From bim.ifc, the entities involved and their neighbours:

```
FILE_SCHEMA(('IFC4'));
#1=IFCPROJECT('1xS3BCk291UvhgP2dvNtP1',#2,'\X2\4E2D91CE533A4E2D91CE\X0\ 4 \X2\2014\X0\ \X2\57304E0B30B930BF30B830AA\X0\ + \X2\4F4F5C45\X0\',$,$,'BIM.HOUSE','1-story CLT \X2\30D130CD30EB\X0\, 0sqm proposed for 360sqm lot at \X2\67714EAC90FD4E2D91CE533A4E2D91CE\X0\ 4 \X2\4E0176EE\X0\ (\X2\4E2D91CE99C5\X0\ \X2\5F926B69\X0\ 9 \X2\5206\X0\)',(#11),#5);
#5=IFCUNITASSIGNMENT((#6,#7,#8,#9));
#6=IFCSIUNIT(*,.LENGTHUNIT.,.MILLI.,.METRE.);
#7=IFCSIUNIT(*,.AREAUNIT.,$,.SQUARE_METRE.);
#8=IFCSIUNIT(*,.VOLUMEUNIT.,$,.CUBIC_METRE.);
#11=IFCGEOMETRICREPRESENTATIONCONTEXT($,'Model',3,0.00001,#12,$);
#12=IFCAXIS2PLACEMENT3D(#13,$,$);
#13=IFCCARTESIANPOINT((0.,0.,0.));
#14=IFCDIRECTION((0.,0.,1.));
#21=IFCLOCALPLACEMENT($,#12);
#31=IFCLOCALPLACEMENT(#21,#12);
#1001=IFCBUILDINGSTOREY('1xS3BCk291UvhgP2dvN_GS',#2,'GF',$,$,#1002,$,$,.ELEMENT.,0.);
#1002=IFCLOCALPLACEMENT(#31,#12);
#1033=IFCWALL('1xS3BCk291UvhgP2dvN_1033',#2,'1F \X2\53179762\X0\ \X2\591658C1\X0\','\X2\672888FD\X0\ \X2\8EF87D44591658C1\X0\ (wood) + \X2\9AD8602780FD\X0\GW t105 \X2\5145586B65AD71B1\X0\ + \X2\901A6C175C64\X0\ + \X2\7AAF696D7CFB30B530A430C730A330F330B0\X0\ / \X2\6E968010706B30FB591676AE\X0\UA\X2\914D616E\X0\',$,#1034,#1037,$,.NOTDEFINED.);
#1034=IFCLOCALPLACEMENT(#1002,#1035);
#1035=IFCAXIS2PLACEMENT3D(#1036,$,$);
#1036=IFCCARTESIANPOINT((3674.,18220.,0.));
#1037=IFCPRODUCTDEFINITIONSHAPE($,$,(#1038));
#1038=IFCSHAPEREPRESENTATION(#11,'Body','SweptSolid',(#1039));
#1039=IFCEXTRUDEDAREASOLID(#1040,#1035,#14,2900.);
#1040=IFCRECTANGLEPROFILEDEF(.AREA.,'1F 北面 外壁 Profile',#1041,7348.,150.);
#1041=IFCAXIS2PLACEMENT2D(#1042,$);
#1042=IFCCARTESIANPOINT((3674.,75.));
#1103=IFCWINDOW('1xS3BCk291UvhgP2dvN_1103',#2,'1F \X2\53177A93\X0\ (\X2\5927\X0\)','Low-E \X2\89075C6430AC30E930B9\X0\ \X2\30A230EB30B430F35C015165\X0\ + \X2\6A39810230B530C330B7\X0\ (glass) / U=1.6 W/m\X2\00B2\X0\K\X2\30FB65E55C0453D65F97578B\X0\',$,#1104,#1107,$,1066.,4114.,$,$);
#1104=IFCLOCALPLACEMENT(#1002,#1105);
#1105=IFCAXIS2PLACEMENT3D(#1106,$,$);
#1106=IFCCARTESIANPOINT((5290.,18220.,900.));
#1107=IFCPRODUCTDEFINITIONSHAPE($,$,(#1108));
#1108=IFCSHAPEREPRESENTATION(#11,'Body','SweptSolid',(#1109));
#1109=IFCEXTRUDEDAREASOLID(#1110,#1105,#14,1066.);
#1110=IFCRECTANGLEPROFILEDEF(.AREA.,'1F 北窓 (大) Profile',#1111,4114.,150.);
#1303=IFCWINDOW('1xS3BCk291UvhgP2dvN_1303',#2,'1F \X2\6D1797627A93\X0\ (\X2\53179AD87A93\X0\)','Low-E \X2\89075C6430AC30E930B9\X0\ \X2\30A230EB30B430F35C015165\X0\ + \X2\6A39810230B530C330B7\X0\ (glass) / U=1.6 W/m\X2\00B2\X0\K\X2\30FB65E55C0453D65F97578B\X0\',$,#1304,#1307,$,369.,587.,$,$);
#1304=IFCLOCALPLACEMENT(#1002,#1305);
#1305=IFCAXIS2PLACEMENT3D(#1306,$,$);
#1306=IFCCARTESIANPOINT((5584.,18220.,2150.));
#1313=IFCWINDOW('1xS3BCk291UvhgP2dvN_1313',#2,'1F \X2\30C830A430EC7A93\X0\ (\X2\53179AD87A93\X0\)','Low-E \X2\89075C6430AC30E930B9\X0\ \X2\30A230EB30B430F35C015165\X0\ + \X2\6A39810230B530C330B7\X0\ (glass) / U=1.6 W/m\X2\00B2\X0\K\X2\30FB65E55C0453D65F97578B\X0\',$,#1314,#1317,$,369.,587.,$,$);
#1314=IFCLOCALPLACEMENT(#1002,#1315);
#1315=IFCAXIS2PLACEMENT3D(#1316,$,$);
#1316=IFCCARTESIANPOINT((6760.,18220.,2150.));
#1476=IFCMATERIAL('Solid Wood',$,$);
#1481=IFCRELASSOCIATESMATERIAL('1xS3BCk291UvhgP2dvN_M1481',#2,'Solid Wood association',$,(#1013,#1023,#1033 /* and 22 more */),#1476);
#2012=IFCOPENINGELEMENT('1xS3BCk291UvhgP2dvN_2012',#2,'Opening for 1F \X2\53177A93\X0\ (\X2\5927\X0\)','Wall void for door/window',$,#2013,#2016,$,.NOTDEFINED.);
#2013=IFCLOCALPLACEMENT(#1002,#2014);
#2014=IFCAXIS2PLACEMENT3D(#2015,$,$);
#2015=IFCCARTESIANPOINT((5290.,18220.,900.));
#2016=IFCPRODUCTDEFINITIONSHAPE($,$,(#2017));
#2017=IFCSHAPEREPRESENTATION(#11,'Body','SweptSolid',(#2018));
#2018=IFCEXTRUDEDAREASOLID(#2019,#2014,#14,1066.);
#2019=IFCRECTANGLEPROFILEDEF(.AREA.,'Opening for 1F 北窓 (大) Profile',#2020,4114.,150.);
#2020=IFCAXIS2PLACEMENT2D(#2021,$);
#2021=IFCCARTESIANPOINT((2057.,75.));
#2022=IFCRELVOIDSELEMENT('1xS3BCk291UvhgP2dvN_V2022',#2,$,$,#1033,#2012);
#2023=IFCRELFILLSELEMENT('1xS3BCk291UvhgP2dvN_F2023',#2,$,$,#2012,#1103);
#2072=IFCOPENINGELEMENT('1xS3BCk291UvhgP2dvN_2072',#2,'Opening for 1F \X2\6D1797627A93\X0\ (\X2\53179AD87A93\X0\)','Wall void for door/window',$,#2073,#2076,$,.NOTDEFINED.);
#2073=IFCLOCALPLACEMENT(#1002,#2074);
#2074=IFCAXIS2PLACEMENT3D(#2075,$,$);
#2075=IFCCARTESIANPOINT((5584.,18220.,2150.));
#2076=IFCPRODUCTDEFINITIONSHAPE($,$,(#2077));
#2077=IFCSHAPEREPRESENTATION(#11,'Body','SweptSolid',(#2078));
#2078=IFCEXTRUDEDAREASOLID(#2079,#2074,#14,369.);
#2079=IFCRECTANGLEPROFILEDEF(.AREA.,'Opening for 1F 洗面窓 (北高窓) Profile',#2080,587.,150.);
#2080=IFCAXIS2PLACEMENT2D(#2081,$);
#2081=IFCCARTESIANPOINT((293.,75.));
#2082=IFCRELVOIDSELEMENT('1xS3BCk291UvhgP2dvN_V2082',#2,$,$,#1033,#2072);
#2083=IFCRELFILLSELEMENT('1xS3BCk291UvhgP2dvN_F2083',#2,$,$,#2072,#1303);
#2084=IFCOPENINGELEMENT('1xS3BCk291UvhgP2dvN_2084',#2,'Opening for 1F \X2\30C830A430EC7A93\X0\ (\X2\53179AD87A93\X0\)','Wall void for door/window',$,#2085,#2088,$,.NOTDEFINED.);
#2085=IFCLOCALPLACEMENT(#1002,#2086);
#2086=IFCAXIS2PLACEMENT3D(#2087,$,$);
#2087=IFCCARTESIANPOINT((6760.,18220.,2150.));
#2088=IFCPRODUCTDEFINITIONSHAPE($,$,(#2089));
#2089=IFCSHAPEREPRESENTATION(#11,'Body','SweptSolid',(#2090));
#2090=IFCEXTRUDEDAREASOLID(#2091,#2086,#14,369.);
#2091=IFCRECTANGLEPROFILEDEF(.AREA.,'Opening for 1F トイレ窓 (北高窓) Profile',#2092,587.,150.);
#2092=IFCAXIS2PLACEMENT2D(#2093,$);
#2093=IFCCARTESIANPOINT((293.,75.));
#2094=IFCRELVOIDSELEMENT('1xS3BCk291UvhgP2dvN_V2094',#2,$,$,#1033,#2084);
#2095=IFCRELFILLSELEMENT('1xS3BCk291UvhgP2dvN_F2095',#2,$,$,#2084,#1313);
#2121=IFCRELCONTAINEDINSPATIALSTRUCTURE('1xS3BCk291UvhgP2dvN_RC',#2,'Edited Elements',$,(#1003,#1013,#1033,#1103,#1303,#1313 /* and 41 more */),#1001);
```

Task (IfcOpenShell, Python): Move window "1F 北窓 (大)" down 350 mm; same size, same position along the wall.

```python
import numpy as np
import ifcopenshell
import ifcopenshell.api.geometry
import ifcopenshell.util.placement
import ifcopenshell.util.unit

model = ifcopenshell.open("bim.ifc")
unit_scale = ifcopenshell.util.unit.calculate_unit_scale(model)

window = model.by_guid("1xS3BCk291UvhgP2dvN_1103")
opening = window.FillsVoids[0].RelatingOpeningElement
dz = -350.0

shift = np.array([0.0, 0.0, dz])
# The window is not placed relative to its opening, so move both.
for product in (opening, window):
    matrix = ifcopenshell.util.placement.get_local_placement(product.ObjectPlacement)
    matrix[:3, 3] += shift
    ifcopenshell.api.geometry.edit_object_placement(model, product=product, matrix=matrix, is_si=False)

print(f"moved by {dz * unit_scale:+.3f} m")

model.write("bim-out.ifc")
```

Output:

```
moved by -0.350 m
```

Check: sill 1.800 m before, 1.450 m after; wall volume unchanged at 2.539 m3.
